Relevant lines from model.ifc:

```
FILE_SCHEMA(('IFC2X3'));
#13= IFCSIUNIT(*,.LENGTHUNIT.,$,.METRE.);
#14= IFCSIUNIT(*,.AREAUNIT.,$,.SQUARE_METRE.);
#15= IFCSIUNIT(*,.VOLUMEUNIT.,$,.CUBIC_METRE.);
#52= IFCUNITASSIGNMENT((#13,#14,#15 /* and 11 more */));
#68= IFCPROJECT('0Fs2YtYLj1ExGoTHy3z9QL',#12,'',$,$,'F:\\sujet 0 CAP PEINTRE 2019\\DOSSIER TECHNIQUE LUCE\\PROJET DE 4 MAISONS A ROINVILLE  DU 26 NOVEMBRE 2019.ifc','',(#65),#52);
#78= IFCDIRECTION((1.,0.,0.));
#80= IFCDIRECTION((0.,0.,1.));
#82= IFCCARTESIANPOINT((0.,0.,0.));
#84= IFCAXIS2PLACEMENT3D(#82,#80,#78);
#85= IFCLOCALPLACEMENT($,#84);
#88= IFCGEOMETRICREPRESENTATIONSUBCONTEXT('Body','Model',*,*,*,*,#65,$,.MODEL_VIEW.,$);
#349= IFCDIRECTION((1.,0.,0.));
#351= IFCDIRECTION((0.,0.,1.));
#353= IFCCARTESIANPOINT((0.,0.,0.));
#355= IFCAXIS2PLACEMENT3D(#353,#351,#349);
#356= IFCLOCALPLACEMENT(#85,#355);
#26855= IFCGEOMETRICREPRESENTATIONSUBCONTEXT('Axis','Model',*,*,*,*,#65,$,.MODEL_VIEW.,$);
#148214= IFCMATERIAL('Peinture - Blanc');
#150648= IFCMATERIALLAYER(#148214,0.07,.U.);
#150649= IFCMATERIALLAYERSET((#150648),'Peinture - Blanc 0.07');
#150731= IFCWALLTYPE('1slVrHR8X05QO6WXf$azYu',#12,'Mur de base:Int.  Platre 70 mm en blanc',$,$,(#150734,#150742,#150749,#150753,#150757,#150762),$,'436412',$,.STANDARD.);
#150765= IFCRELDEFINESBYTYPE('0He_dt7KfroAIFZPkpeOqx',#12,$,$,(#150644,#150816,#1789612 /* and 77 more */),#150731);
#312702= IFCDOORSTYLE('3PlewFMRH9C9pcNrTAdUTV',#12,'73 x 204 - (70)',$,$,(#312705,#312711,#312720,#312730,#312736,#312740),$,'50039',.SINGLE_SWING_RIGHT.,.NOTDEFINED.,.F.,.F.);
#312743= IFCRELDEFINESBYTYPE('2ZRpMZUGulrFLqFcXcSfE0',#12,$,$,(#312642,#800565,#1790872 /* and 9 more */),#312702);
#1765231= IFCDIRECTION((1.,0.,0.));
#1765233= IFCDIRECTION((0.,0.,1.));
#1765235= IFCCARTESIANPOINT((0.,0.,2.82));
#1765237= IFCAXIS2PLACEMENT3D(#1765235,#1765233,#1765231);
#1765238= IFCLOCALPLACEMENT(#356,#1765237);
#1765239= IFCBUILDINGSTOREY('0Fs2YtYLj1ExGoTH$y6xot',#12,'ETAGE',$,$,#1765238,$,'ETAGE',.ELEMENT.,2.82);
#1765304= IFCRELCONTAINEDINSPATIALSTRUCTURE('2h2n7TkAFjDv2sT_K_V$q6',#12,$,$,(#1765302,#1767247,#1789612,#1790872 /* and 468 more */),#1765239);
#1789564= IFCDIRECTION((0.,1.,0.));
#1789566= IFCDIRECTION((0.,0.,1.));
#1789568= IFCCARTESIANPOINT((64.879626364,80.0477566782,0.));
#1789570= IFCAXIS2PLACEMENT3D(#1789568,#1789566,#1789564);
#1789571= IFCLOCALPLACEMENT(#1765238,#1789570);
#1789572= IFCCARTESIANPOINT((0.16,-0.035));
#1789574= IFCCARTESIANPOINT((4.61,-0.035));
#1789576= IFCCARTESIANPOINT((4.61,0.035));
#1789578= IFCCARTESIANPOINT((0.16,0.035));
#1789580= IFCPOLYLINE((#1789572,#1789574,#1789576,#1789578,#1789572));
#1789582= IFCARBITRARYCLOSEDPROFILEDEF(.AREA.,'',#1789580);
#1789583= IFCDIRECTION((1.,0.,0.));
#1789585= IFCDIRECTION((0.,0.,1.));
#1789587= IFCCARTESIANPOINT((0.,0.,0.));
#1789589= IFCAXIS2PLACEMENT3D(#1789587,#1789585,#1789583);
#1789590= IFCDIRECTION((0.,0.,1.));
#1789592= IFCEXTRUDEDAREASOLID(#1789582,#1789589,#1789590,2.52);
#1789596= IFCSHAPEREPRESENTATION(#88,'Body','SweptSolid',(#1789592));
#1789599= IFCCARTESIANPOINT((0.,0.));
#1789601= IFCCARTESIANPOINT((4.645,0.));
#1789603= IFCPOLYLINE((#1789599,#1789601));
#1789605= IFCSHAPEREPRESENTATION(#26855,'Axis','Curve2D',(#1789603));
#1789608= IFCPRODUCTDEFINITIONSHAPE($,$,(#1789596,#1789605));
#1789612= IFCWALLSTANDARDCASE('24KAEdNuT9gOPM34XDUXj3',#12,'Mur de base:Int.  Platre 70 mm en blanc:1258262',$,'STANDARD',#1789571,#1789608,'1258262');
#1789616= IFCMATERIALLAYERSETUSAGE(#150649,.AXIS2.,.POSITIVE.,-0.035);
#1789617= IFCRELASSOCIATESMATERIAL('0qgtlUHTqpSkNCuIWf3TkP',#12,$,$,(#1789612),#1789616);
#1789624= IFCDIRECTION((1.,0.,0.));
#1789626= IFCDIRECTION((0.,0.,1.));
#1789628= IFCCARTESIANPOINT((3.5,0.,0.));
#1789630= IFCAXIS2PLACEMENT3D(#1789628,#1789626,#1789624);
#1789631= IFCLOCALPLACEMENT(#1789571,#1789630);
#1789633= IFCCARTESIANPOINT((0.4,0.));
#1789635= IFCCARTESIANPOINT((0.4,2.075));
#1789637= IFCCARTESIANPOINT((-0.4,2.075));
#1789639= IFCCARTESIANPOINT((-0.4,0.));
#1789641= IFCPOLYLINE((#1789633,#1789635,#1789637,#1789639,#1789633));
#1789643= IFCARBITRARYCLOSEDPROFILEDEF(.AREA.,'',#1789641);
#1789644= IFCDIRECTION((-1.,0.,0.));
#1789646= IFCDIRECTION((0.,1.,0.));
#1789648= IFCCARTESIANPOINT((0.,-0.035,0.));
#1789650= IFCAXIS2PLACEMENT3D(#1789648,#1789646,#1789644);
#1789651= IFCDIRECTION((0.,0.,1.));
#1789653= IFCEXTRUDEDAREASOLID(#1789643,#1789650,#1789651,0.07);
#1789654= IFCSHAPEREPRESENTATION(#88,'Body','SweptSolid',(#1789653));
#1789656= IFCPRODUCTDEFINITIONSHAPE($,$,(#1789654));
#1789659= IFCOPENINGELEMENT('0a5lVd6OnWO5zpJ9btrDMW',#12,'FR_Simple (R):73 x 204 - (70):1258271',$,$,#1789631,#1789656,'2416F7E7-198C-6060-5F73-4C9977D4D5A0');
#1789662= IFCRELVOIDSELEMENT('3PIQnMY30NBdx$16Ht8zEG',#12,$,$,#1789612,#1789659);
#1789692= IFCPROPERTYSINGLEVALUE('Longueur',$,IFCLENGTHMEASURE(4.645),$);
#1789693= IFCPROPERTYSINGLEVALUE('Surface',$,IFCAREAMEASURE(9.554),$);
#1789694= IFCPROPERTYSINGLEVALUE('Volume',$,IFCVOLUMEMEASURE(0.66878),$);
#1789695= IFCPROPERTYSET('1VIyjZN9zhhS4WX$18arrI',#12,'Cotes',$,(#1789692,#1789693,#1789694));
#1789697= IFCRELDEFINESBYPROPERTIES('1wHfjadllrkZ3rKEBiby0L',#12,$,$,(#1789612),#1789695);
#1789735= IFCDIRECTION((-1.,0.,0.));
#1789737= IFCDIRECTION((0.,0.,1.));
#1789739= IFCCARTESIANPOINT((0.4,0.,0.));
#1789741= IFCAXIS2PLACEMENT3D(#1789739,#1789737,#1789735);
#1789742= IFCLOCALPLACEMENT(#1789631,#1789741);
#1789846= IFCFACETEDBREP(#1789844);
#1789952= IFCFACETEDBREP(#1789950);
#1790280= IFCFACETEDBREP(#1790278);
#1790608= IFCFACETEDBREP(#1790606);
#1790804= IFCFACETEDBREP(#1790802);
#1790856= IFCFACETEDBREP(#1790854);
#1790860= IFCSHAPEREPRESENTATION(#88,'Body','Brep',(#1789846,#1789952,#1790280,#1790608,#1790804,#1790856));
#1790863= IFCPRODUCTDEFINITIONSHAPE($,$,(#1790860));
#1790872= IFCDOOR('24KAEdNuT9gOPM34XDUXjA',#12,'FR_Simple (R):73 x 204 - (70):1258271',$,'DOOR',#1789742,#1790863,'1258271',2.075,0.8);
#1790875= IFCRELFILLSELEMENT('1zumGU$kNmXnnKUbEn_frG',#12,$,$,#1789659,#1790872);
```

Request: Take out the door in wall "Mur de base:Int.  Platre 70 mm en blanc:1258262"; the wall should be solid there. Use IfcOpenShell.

```python
import ifcopenshell
import ifcopenshell.api.feature
import ifcopenshell.api.pset
import ifcopenshell.api.root
import ifcopenshell.geom
import ifcopenshell.util.element
import ifcopenshell.util.shape
import ifcopenshell.util.unit

model = ifcopenshell.open("model.ifc")
area_scale = ifcopenshell.util.unit.calculate_unit_scale(model, "AREAUNIT")
volume_scale = ifcopenshell.util.unit.calculate_unit_scale(model, "VOLUMEUNIT")
settings = ifcopenshell.geom.settings()


def volume(element):
    """Net volume in cubic metres, openings subtracted."""
    shape = ifcopenshell.geom.create_shape(settings, element)
    return ifcopenshell.util.shape.get_volume(shape.geometry)


door = model.by_id(1790872)
opening = door.FillsVoids[0].RelatingOpeningElement
wall = opening.VoidsElements[0].RelatingBuildingElement
before = volume(wall)

ifcopenshell.api.root.remove_product(model, product=door)
ifcopenshell.api.feature.remove_feature(model, feature=opening)

after = volume(wall)
thickness = 0.07  # wall thickness in metres

# Update the wall's stored quantities.
pset = model.by_id(ifcopenshell.util.element.get_pset(wall, "Cotes", should_inherit=False)["id"])
ifcopenshell.api.pset.edit_pset(model, pset=pset, properties={
    "Surface": model.create_entity("IfcAreaMeasure", after / thickness / area_scale),
    "Volume": model.create_entity("IfcVolumeMeasure", after / volume_scale),
})

print(f"wall volume {before:.3f} -> {after:.3f} m3")

model.write("model_updated.ifc")
```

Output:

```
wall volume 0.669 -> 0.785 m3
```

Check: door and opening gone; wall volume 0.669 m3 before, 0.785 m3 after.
